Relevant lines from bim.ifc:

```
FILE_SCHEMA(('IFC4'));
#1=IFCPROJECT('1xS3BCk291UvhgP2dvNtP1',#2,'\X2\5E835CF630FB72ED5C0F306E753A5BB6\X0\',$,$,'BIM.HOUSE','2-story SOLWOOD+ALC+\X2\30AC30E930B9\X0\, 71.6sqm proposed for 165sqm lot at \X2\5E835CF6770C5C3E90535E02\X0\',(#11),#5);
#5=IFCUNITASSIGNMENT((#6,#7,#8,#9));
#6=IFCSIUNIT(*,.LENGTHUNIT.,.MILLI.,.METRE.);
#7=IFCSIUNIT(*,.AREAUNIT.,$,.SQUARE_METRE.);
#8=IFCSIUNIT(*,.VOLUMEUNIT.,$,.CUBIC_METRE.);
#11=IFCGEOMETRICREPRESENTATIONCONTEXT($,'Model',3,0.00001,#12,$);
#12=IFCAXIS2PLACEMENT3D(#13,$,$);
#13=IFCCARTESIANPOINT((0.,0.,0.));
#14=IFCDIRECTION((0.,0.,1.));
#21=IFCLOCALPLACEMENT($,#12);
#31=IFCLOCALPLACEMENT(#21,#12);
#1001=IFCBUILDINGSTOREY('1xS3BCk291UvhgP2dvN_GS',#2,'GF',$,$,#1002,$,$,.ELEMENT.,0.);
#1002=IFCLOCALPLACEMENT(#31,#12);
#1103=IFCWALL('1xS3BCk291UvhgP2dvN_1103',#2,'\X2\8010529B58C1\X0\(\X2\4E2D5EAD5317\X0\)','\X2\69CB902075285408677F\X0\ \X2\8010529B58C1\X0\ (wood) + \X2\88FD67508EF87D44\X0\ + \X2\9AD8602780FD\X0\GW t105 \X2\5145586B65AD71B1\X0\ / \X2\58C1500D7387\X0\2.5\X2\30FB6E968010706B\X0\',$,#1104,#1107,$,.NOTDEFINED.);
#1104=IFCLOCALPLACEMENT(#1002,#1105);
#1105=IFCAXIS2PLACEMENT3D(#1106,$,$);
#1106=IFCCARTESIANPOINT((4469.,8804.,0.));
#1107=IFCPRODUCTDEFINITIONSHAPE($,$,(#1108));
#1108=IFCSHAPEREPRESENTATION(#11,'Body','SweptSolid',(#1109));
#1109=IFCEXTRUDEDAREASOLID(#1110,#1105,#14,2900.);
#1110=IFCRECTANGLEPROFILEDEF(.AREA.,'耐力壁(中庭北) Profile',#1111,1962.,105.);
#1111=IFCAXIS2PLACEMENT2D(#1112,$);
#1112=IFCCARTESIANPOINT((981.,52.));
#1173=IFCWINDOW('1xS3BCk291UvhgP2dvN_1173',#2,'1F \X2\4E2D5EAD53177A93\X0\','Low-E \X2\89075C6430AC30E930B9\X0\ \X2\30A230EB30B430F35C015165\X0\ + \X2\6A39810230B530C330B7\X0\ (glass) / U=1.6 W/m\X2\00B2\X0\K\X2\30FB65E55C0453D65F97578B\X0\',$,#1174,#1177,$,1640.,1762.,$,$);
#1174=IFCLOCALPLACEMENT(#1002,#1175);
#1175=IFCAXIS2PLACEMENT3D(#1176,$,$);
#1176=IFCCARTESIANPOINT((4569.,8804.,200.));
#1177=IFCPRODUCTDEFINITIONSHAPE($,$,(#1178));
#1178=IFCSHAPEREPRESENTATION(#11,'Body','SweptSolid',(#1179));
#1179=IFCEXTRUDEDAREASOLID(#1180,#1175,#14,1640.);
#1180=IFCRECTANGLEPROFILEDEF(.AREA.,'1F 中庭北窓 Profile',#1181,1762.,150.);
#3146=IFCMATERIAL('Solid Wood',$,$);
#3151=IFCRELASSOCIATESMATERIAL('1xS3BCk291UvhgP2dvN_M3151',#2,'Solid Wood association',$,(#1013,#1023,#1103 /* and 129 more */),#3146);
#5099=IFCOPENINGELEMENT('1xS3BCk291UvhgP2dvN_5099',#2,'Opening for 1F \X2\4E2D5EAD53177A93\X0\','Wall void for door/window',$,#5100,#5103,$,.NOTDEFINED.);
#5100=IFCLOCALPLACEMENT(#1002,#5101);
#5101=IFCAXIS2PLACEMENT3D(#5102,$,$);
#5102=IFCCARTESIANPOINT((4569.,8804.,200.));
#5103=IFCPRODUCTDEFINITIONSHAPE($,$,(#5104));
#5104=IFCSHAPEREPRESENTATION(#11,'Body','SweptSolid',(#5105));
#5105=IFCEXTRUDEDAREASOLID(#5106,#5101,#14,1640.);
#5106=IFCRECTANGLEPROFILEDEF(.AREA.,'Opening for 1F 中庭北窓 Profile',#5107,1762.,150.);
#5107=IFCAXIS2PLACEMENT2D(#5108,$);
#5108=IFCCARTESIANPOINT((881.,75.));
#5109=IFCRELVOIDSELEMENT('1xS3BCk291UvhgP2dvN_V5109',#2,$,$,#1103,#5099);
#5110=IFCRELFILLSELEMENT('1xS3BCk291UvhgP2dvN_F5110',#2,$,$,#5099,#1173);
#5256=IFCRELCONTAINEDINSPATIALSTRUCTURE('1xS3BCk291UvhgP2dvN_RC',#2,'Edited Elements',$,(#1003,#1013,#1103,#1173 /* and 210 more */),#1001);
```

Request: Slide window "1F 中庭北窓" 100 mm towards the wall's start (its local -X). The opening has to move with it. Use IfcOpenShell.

```python
import ifcopenshell
import ifcopenshell.api.geometry
import ifcopenshell.util.placement

model = ifcopenshell.open("bim.ifc")

window = model.by_guid("1xS3BCk291UvhgP2dvN_1173")
opening = window.FillsVoids[0].RelatingOpeningElement
wall = opening.VoidsElements[0].RelatingBuildingElement

wall_matrix = ifcopenshell.util.placement.get_local_placement(wall.ObjectPlacement)
shift = wall_matrix[:3, 0] * -100.0
before = ifcopenshell.util.placement.get_local_placement(window.ObjectPlacement)[:3, 3].copy()

# The window is not placed relative to its opening, so move both.
for product in (opening, window):
    matrix = ifcopenshell.util.placement.get_local_placement(product.ObjectPlacement)
    matrix[:3, 3] += shift
    ifcopenshell.api.geometry.edit_object_placement(model, product=product, matrix=matrix, is_si=False)

after = ifcopenshell.util.placement.get_local_placement(window.ObjectPlacement)[:3, 3]
print("window moved by", (after - before).round(3) + 0.0)

model.write("bim_edited.ifc")
```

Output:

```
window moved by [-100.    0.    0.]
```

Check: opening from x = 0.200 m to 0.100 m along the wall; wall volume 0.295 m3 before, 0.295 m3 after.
